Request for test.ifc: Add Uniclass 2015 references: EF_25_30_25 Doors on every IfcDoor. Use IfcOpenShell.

First a look at what the model holds.

```python
import ifcopenshell

model = ifcopenshell.open("test.ifc")
print(model.schema)
print("classifications:", [c.Name for c in model.by_type("IfcClassification")])
for ifc_class in ("IfcDoor", "IfcRoof", "IfcStair", "IfcWall", "IfcWindow"):
    print(ifc_class, len(model.by_type(ifc_class)))
```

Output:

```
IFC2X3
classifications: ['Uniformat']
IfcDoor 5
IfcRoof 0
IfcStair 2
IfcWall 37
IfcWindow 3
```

```python
import ifcopenshell
import ifcopenshell.api.classification

model = ifcopenshell.open("test.ifc")

# IFC2X3 requires Source and Edition and has no link from the project to the system.
system = model.create_entity("IfcClassification", Source="NBS", Edition="2015", Name="Uniclass 2015")

codes = {
    "IfcDoor": ("EF_25_30_25", "Doors"),
}
for ifc_class, (code, name) in codes.items():
    products = model.by_type(ifc_class)
    ifcopenshell.api.classification.add_reference(
        model, products=products, classification=system, identification=code, name=name
    )
    print(code, len(products))

model.write("test_edited.ifc")
```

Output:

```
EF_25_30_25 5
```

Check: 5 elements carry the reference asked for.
